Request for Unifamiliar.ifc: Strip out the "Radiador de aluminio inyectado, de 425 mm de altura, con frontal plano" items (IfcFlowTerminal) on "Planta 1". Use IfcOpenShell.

First a look at what the model holds.

```python
import ifcopenshell
import ifcopenshell.util.element

model = ifcopenshell.open("Unifamiliar.ifc")
print(model.schema)
storey = next(s for s in model.by_type("IfcBuildingStorey") if s.Name == "Planta 1")
terminals = [e for e in ifcopenshell.util.element.get_decomposition(storey) if e.is_a("IfcFlowTerminal")]
seen = {}
for e in terminals:
    element_type = ifcopenshell.util.element.get_type(e)
    name = element_type.Name if element_type not in (None, e) else None
    seen[name] = seen.get(name, 0) + 1
for name, count in sorted(seen.items(), key=str):
    print(count, "x", name)
```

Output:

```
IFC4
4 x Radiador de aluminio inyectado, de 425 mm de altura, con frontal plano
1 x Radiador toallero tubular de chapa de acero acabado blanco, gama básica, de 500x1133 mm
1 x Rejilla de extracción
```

```python
import ifcopenshell
import ifcopenshell.api.root
import ifcopenshell.util.element

model = ifcopenshell.open("Unifamiliar.ifc")

storey = next(s for s in model.by_type("IfcBuildingStorey") if s.Name == "Planta 1")
terminals = [e for e in ifcopenshell.util.element.get_decomposition(storey) if e.is_a("IfcFlowTerminal")]
targets = [e for e in terminals if (t := ifcopenshell.util.element.get_type(e)) not in (None, e) and t.Name == "Radiador de aluminio inyectado, de 425 mm de altura, con frontal plano"]

for e in targets:
    ifcopenshell.api.root.remove_product(model, product=e)
print(len(targets), "removed")

model.write("Unifamiliar_v2.ifc")
```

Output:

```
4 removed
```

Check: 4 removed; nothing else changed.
